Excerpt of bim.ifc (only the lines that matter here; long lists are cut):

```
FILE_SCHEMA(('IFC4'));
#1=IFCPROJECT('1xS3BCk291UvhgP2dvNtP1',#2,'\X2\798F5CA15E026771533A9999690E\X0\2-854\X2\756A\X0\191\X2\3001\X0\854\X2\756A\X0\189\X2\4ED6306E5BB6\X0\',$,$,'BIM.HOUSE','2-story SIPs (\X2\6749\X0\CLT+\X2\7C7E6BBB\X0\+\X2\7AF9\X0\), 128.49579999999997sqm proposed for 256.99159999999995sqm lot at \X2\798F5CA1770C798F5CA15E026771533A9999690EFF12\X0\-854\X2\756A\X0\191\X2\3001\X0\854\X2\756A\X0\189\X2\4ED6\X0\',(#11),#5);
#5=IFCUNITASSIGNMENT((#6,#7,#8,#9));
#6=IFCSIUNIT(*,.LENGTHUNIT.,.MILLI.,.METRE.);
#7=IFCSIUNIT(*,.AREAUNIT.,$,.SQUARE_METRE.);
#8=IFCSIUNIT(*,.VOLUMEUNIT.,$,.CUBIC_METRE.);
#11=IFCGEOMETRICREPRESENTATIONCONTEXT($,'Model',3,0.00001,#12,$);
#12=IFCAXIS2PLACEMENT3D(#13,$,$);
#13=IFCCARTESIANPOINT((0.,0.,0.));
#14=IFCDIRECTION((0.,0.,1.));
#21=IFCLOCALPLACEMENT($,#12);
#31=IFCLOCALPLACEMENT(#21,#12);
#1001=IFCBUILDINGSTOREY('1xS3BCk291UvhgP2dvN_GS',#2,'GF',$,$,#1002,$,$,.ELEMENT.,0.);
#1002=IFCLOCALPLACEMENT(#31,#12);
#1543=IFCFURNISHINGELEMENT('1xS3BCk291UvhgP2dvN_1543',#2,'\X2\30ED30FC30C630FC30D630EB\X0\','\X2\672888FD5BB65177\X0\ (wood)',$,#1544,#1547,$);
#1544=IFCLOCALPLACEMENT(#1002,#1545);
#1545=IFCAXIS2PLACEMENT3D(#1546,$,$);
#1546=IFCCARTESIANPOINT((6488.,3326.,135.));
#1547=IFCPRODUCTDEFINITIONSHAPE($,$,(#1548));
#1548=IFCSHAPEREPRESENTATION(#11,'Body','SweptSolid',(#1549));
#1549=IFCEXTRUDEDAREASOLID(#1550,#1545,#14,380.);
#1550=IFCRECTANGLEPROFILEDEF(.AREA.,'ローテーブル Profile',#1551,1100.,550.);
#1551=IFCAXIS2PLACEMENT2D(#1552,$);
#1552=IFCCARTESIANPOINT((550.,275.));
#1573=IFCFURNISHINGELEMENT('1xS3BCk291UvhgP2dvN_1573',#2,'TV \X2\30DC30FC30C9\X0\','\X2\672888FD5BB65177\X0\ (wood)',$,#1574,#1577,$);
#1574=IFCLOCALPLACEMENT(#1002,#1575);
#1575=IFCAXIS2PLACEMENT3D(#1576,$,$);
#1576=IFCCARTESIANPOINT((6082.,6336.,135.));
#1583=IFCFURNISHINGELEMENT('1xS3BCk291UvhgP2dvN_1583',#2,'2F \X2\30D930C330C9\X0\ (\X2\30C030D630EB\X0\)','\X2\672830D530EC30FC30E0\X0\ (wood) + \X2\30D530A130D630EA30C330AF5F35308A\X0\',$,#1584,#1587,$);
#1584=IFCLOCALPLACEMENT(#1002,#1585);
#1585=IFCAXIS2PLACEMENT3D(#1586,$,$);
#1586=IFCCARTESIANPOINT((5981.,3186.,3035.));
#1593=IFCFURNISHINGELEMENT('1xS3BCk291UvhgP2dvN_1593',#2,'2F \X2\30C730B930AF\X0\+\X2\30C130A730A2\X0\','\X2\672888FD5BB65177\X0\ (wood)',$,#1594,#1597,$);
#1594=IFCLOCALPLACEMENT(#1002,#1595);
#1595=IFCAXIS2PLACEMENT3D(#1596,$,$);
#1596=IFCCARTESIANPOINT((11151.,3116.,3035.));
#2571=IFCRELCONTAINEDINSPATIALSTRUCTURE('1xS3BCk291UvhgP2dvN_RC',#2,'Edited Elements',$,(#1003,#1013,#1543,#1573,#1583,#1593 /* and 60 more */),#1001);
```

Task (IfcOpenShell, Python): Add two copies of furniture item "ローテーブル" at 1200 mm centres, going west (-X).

```python
import numpy as np
import ifcopenshell
import ifcopenshell.api.geometry
import ifcopenshell.api.root
import ifcopenshell.util.element
import ifcopenshell.util.placement

model = ifcopenshell.open("bim.ifc")


def reuse_history(source, copy):
    """copy_class also copies each property set's owner history, people and application; keep the originals."""
    for rel in copy.IsDefinedBy:
        if rel.is_a("IfcRelDefinesByProperties") and (history := rel.RelatingPropertyDefinition.OwnerHistory):
            rel.RelatingPropertyDefinition.OwnerHistory = source.OwnerHistory
            ifcopenshell.util.element.remove_deep2(model, history)


source = model.by_guid("1xS3BCk291UvhgP2dvN_1543")
base = ifcopenshell.util.placement.get_local_placement(source.ObjectPlacement)
step = np.array([-1.0, 0.0, 0.0]) * 1200.0

for i in range(1, 3):
    copy = ifcopenshell.api.root.copy_class(model, product=source)
    copy.Representation = ifcopenshell.util.element.copy_deep(
        model, source.Representation, exclude=["IfcGeometricRepresentationContext", "IfcRepresentationMap"]
    )
    reuse_history(source, copy)
    matrix = base.copy()
    matrix[:3, 3] += i * step
    print("added at", matrix[:3, 3].round(3) + 0.0)
    ifcopenshell.api.geometry.edit_object_placement(model, product=copy, matrix=matrix, is_si=False)

model.write("bim_edited.ifc")
```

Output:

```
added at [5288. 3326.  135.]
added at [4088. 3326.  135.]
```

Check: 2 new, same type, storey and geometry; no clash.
